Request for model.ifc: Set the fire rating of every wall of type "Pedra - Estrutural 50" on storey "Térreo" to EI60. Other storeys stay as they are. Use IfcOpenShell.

First a look at what the model holds.

```python
import ifcopenshell
import ifcopenshell.util.element

model = ifcopenshell.open("model.ifc")
print(model.schema)
storey = next(s for s in model.by_type("IfcBuildingStorey") if s.Name == "Térreo")
walls = [e for e in ifcopenshell.util.element.get_decomposition(storey) if e.is_a("IfcWall")]
seen = {}
for e in walls:
    element_type = ifcopenshell.util.element.get_type(e)
    key = (element_type.Name if element_type != e and element_type else None, ifcopenshell.util.element.get_pset(e, "Pset_WallCommon", "FireRating"))
    seen[key] = seen.get(key, 0) + 1
for (name, value), count in sorted(seen.items(), key=str):
    print(count, "x", name, "|", value)
```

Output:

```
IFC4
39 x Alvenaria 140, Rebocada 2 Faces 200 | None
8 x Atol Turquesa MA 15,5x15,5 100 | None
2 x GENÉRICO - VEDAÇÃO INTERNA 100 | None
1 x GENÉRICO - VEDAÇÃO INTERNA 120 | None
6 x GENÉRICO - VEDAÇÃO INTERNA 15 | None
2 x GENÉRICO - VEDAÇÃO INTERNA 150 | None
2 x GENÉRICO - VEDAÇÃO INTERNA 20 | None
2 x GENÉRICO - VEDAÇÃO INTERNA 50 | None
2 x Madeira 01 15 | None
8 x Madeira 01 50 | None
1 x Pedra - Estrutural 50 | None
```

```python
import ifcopenshell
import ifcopenshell.api.pset
import ifcopenshell.util.element

model = ifcopenshell.open("model.ifc")

storey = next(s for s in model.by_type("IfcBuildingStorey") if s.Name == "Térreo")
walls = [e for e in ifcopenshell.util.element.get_decomposition(storey) if e.is_a("IfcWall")]

count = 0
for e in walls:
    element_type = ifcopenshell.util.element.get_type(e)
    if element_type in (None, e) or element_type.Name != "Pedra - Estrutural 50":
        continue
    # add_pset returns the element's existing set when there is one.
    pset = ifcopenshell.api.pset.add_pset(model, product=e, name="Pset_WallCommon")
    ifcopenshell.api.pset.edit_pset(model, pset=pset, properties={"FireRating": "EI60"})
    count += 1

print(count, "walls updated")

model.write("model_edited.ifc")
```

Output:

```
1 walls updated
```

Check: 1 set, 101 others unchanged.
